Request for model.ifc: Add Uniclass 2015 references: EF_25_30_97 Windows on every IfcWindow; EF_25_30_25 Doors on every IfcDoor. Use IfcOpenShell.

First a look at what the model holds.

```python
import ifcopenshell

model = ifcopenshell.open("model.ifc")
print(model.schema)
print("classifications:", [c.Name for c in model.by_type("IfcClassification")])
for ifc_class in ("IfcDoor", "IfcRoof", "IfcStair", "IfcWall", "IfcWindow"):
    print(ifc_class, len(model.by_type(ifc_class)))
```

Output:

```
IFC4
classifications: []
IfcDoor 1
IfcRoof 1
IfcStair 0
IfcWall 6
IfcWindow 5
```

```python
import ifcopenshell
import ifcopenshell.api.classification

model = ifcopenshell.open("model.ifc")

system = ifcopenshell.api.classification.add_classification(model, classification="Uniclass 2015")

codes = {
    "IfcWindow": ("EF_25_30_97", "Windows"),
    "IfcDoor": ("EF_25_30_25", "Doors"),
}
for ifc_class, (code, name) in codes.items():
    products = model.by_type(ifc_class)
    ifcopenshell.api.classification.add_reference(
        model, products=products, classification=system, identification=code, name=name
    )
    print(code, len(products))

model.write("model_rev.ifc")
```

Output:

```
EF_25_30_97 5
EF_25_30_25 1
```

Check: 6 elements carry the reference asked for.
